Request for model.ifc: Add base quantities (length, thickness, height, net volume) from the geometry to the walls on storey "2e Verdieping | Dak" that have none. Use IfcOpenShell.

First a look at what the model holds.

```python
import ifcopenshell
import ifcopenshell.util.element
import ifcopenshell.util.unit

model = ifcopenshell.open("model.ifc")
print(model.schema)
for unit_type in ("LENGTHUNIT", "AREAUNIT", "VOLUMEUNIT"):
    print(unit_type, ifcopenshell.util.unit.calculate_unit_scale(model, unit_type))
storey = next(s for s in model.by_type("IfcBuildingStorey") if s.Name == "2e Verdieping | Dak")
walls = [e for e in ifcopenshell.util.element.get_decomposition(storey) if e.is_a("IfcWall")]
for e in sorted(walls, key=lambda e: e.id()):
    print(e.id(), e.is_a(), e.Name, list(ifcopenshell.util.element.get_psets(e, qtos_only=True)), sep=" | ")
```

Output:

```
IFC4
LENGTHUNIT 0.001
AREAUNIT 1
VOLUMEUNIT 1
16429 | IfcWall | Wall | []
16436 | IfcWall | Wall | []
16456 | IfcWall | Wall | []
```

```python
import ifcopenshell
import ifcopenshell.api.pset
import ifcopenshell.geom
import ifcopenshell.util.element
import ifcopenshell.util.shape
import ifcopenshell.util.unit

model = ifcopenshell.open("model.ifc")
unit_scale = ifcopenshell.util.unit.calculate_unit_scale(model)
volume_scale = ifcopenshell.util.unit.calculate_unit_scale(model, "VOLUMEUNIT")
settings = ifcopenshell.geom.settings()

storey = next(s for s in model.by_type("IfcBuildingStorey") if s.Name == "2e Verdieping | Dak")
walls = [e for e in ifcopenshell.util.element.get_decomposition(storey) if e.is_a("IfcWall")]

for e in sorted(walls, key=lambda e: e.id()):
    if ifcopenshell.util.element.get_psets(e, qtos_only=True, should_inherit=False):
        continue
    # Geometry comes back in metres, in the element's own axes.
    shape = ifcopenshell.geom.create_shape(settings, e)
    values = {
        "Length": ifcopenshell.util.shape.get_x(shape.geometry) / unit_scale,
        "Width": ifcopenshell.util.shape.get_y(shape.geometry) / unit_scale,
        "Height": ifcopenshell.util.shape.get_z(shape.geometry) / unit_scale,
        "NetVolume": ifcopenshell.util.shape.get_volume(shape.geometry) / volume_scale,
    }
    qto = ifcopenshell.api.pset.add_qto(model, product=e, name="Qto_WallBaseQuantities")
    ifcopenshell.api.pset.edit_qto(model, qto=qto, properties=values)
    print(e.id(), {k: round(v, 3) for k, v in values.items()})

model.write("model_rev.ifc")
```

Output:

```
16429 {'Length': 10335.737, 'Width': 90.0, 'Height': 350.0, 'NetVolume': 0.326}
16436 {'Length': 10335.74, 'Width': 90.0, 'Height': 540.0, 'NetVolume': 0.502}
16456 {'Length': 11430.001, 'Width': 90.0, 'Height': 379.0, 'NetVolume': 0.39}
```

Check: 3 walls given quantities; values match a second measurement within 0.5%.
